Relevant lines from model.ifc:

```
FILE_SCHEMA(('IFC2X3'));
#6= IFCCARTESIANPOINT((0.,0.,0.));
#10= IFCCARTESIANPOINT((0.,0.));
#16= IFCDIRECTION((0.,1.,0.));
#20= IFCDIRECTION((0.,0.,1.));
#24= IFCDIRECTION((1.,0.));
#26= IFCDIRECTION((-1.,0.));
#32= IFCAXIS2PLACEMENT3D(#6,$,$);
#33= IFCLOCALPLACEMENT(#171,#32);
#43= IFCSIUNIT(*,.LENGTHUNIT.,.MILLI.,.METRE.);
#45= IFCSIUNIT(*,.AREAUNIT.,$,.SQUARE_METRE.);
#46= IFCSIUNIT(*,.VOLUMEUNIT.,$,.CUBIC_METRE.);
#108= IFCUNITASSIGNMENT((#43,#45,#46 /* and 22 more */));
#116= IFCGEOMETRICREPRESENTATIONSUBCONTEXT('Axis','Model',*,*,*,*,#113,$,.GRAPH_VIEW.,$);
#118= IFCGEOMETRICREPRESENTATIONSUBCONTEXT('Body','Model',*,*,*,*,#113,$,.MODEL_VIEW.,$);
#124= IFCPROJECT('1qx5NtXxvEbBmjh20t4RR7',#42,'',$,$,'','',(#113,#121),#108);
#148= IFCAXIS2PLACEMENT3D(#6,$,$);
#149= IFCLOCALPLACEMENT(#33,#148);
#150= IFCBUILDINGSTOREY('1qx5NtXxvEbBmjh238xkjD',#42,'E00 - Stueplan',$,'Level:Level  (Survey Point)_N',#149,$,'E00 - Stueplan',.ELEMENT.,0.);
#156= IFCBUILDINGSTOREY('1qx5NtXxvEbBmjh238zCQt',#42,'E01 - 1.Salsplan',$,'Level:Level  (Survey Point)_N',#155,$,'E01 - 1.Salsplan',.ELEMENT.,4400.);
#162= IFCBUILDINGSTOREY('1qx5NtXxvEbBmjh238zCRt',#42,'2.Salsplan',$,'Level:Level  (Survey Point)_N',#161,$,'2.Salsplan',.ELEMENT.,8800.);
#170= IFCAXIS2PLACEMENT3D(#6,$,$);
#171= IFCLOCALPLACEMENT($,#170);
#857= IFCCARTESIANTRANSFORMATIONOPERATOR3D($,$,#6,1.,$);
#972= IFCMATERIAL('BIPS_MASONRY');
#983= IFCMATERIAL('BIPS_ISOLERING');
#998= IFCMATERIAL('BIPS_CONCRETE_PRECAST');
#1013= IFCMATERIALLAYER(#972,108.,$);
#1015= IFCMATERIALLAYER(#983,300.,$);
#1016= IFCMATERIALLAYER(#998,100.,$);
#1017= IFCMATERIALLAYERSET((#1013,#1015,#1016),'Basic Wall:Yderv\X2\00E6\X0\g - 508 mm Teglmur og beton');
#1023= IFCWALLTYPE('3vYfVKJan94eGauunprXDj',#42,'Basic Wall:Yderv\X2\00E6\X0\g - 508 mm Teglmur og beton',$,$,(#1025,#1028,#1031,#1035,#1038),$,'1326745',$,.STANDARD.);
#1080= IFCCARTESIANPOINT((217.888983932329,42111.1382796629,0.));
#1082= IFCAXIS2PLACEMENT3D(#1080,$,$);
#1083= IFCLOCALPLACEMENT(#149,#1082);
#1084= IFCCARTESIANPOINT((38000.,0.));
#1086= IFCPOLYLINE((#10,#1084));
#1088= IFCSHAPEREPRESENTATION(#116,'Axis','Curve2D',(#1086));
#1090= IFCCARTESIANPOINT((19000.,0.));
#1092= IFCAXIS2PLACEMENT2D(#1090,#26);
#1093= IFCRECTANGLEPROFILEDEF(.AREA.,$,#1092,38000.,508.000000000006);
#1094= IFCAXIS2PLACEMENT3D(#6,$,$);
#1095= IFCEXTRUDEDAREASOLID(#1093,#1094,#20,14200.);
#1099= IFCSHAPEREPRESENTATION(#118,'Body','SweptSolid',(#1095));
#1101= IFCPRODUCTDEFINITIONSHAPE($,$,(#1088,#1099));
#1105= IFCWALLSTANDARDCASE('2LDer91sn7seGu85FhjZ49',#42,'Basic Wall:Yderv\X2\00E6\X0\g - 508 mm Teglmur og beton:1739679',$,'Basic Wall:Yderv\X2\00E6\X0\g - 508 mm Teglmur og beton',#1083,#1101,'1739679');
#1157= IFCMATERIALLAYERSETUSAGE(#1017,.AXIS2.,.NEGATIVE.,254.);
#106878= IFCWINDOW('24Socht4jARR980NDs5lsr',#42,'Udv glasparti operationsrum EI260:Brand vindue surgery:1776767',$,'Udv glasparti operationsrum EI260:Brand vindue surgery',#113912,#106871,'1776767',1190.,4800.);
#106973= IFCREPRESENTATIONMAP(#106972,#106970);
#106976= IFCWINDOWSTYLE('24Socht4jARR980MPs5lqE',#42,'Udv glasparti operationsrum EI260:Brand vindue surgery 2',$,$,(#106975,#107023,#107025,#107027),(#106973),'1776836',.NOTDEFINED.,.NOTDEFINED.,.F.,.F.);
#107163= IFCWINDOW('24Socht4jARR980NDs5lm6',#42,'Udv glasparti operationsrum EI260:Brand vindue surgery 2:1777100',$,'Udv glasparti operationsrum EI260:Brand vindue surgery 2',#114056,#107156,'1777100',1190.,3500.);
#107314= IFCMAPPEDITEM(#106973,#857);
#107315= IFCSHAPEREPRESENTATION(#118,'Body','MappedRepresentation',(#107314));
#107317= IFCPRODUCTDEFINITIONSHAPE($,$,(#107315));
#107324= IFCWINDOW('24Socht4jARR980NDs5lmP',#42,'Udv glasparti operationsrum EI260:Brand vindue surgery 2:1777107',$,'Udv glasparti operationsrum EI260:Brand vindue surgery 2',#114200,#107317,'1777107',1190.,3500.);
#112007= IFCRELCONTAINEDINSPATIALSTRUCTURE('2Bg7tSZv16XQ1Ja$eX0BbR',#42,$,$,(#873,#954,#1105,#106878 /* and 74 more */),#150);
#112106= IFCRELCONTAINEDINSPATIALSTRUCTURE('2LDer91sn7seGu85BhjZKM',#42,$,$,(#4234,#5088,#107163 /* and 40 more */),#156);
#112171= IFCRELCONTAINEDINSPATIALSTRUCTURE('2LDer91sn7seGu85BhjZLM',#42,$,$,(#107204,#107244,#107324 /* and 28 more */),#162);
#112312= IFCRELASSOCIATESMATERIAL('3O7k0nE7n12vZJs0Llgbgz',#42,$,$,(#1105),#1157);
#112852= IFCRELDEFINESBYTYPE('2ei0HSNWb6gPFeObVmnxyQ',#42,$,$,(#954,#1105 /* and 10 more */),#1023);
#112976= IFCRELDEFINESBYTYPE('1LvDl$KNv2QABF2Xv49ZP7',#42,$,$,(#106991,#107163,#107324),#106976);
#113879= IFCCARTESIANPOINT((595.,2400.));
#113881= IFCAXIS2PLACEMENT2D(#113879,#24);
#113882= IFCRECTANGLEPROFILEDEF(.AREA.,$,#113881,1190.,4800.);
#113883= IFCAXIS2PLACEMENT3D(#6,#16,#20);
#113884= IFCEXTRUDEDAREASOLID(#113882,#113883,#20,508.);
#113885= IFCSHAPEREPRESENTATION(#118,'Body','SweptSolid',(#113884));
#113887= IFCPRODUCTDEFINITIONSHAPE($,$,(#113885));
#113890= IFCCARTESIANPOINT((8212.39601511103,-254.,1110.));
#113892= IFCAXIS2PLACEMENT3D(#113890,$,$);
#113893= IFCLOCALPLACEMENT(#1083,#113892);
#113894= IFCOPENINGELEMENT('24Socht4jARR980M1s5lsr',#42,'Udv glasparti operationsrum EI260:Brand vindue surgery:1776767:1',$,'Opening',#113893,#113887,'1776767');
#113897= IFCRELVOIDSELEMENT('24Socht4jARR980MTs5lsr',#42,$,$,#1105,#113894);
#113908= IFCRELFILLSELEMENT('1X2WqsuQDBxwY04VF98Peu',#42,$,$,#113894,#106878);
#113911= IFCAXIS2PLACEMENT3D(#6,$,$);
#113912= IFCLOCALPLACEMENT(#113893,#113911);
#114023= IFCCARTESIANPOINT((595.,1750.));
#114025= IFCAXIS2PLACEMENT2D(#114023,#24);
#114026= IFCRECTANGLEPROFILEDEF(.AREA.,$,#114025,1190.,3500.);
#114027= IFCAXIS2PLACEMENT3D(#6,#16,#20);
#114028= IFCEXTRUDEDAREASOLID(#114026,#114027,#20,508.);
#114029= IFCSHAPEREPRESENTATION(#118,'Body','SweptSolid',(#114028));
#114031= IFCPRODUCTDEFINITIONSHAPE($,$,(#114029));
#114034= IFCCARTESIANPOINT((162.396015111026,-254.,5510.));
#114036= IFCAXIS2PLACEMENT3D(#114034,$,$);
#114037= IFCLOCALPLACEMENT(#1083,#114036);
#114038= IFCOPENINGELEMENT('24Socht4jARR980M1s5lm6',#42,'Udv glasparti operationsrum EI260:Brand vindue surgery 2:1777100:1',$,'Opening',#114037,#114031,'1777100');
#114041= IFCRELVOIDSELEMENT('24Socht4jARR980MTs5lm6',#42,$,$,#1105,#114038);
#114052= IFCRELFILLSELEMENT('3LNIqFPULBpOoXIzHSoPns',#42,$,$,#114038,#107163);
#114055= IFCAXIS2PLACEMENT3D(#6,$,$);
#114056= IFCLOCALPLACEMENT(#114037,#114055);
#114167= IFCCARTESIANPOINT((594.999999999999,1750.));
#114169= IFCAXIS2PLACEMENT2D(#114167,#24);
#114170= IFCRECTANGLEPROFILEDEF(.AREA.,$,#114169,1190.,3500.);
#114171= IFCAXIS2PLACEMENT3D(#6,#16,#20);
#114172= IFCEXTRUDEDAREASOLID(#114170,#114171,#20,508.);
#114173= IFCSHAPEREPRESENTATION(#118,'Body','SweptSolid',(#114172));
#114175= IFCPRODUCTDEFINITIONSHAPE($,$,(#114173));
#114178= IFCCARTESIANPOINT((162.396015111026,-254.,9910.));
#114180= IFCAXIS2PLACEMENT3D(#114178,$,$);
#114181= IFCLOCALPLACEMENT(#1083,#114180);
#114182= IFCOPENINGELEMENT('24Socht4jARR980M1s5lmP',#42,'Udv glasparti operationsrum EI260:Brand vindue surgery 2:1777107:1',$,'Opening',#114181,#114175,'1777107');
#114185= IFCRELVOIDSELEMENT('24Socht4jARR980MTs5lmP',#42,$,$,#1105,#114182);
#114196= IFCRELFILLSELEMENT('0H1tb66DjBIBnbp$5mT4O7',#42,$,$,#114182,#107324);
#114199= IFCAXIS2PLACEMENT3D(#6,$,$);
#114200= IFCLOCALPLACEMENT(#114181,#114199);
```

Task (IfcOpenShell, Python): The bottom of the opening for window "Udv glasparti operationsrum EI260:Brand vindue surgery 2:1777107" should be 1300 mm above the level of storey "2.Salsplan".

```python
import numpy as np
import ifcopenshell
import ifcopenshell.api.geometry
import ifcopenshell.geom
import ifcopenshell.util.element
import ifcopenshell.util.placement
import ifcopenshell.util.shape
import ifcopenshell.util.unit

model = ifcopenshell.open("model.ifc")
unit_scale = ifcopenshell.util.unit.calculate_unit_scale(model)

window = model.by_id(107324)
opening = window.FillsVoids[0].RelatingOpeningElement
storey = ifcopenshell.util.element.get_container(window, ifc_class="IfcBuildingStorey")
level = ifcopenshell.util.placement.get_local_placement(storey.ObjectPlacement)[2, 3]

# The opening's origin need not be at the sill, so measure its lowest point.
shape = ifcopenshell.geom.create_shape(ifcopenshell.geom.settings(), opening)
bottom = ifcopenshell.util.shape.get_shape_bottom_elevation(shape, shape.geometry) / unit_scale
dz = level + 1.3 / unit_scale - bottom

shift = np.array([0.0, 0.0, dz])
# The window is placed relative to its opening, so it follows when the opening moves.
matrix = ifcopenshell.util.placement.get_local_placement(opening.ObjectPlacement)
matrix[:3, 3] += shift
ifcopenshell.api.geometry.edit_object_placement(
    model, product=opening, matrix=matrix, is_si=False, should_transform_children=True
)

print(f"moved by {dz * unit_scale:+.3f} m")

model.write("model-out.ifc")
```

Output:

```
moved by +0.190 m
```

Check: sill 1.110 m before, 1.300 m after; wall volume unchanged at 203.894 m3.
